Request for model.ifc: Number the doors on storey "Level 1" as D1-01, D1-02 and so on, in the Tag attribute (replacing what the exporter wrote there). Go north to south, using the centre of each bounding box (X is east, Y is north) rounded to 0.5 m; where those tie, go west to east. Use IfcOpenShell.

First a look at what the model holds.

```python
import ifcopenshell
import ifcopenshell.util.element
import ifcopenshell.util.placement

model = ifcopenshell.open("model.ifc")
print(model.schema)
storey = next(s for s in model.by_type("IfcBuildingStorey") if s.Name == "Level 1")
doors = [e for e in ifcopenshell.util.element.get_decomposition(storey) if e.is_a("IfcDoor")]
for e in sorted(doors, key=lambda e: e.id()):
    origin = ifcopenshell.util.placement.get_local_placement(e.ObjectPlacement)[:3, 3]
    print(e.id(), e.Tag, e.Name, origin.round(2) + 0.0, sep=" | ")
```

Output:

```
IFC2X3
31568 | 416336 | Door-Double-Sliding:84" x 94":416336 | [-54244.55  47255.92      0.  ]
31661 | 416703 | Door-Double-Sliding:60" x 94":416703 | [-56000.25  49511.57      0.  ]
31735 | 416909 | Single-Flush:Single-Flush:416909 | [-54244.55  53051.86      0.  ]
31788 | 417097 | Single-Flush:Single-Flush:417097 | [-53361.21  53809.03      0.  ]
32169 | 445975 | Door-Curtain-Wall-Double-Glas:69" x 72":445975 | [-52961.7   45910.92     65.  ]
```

```python
import ifcopenshell
import ifcopenshell.geom
import ifcopenshell.util.element
import ifcopenshell.util.shape

model = ifcopenshell.open("model.ifc")
settings = ifcopenshell.geom.settings()
settings.set("use-world-coords", True)


def centre(element):
    shape = ifcopenshell.geom.create_shape(settings, element)
    return ifcopenshell.util.shape.get_bbox_centroid(shape.geometry)


storey = next(s for s in model.by_type("IfcBuildingStorey") if s.Name == "Level 1")
doors = [e for e in ifcopenshell.util.element.get_decomposition(storey) if e.is_a("IfcDoor")]

# Insertion points can sit at a corner or the storey origin, so sort by the geometry (in metres).
centres = {e: centre(e) for e in doors}
doors.sort(key=lambda e: (-round(centres[e][1] / 0.5), centres[e][0]))

for i, e in enumerate(doors, start=1):
    number = f"D1-{i:02d}"
    e.Tag = number
    print(e.id(), number)

model.write("model-out.ifc")
```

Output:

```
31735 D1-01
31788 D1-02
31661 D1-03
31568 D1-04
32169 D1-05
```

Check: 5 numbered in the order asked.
